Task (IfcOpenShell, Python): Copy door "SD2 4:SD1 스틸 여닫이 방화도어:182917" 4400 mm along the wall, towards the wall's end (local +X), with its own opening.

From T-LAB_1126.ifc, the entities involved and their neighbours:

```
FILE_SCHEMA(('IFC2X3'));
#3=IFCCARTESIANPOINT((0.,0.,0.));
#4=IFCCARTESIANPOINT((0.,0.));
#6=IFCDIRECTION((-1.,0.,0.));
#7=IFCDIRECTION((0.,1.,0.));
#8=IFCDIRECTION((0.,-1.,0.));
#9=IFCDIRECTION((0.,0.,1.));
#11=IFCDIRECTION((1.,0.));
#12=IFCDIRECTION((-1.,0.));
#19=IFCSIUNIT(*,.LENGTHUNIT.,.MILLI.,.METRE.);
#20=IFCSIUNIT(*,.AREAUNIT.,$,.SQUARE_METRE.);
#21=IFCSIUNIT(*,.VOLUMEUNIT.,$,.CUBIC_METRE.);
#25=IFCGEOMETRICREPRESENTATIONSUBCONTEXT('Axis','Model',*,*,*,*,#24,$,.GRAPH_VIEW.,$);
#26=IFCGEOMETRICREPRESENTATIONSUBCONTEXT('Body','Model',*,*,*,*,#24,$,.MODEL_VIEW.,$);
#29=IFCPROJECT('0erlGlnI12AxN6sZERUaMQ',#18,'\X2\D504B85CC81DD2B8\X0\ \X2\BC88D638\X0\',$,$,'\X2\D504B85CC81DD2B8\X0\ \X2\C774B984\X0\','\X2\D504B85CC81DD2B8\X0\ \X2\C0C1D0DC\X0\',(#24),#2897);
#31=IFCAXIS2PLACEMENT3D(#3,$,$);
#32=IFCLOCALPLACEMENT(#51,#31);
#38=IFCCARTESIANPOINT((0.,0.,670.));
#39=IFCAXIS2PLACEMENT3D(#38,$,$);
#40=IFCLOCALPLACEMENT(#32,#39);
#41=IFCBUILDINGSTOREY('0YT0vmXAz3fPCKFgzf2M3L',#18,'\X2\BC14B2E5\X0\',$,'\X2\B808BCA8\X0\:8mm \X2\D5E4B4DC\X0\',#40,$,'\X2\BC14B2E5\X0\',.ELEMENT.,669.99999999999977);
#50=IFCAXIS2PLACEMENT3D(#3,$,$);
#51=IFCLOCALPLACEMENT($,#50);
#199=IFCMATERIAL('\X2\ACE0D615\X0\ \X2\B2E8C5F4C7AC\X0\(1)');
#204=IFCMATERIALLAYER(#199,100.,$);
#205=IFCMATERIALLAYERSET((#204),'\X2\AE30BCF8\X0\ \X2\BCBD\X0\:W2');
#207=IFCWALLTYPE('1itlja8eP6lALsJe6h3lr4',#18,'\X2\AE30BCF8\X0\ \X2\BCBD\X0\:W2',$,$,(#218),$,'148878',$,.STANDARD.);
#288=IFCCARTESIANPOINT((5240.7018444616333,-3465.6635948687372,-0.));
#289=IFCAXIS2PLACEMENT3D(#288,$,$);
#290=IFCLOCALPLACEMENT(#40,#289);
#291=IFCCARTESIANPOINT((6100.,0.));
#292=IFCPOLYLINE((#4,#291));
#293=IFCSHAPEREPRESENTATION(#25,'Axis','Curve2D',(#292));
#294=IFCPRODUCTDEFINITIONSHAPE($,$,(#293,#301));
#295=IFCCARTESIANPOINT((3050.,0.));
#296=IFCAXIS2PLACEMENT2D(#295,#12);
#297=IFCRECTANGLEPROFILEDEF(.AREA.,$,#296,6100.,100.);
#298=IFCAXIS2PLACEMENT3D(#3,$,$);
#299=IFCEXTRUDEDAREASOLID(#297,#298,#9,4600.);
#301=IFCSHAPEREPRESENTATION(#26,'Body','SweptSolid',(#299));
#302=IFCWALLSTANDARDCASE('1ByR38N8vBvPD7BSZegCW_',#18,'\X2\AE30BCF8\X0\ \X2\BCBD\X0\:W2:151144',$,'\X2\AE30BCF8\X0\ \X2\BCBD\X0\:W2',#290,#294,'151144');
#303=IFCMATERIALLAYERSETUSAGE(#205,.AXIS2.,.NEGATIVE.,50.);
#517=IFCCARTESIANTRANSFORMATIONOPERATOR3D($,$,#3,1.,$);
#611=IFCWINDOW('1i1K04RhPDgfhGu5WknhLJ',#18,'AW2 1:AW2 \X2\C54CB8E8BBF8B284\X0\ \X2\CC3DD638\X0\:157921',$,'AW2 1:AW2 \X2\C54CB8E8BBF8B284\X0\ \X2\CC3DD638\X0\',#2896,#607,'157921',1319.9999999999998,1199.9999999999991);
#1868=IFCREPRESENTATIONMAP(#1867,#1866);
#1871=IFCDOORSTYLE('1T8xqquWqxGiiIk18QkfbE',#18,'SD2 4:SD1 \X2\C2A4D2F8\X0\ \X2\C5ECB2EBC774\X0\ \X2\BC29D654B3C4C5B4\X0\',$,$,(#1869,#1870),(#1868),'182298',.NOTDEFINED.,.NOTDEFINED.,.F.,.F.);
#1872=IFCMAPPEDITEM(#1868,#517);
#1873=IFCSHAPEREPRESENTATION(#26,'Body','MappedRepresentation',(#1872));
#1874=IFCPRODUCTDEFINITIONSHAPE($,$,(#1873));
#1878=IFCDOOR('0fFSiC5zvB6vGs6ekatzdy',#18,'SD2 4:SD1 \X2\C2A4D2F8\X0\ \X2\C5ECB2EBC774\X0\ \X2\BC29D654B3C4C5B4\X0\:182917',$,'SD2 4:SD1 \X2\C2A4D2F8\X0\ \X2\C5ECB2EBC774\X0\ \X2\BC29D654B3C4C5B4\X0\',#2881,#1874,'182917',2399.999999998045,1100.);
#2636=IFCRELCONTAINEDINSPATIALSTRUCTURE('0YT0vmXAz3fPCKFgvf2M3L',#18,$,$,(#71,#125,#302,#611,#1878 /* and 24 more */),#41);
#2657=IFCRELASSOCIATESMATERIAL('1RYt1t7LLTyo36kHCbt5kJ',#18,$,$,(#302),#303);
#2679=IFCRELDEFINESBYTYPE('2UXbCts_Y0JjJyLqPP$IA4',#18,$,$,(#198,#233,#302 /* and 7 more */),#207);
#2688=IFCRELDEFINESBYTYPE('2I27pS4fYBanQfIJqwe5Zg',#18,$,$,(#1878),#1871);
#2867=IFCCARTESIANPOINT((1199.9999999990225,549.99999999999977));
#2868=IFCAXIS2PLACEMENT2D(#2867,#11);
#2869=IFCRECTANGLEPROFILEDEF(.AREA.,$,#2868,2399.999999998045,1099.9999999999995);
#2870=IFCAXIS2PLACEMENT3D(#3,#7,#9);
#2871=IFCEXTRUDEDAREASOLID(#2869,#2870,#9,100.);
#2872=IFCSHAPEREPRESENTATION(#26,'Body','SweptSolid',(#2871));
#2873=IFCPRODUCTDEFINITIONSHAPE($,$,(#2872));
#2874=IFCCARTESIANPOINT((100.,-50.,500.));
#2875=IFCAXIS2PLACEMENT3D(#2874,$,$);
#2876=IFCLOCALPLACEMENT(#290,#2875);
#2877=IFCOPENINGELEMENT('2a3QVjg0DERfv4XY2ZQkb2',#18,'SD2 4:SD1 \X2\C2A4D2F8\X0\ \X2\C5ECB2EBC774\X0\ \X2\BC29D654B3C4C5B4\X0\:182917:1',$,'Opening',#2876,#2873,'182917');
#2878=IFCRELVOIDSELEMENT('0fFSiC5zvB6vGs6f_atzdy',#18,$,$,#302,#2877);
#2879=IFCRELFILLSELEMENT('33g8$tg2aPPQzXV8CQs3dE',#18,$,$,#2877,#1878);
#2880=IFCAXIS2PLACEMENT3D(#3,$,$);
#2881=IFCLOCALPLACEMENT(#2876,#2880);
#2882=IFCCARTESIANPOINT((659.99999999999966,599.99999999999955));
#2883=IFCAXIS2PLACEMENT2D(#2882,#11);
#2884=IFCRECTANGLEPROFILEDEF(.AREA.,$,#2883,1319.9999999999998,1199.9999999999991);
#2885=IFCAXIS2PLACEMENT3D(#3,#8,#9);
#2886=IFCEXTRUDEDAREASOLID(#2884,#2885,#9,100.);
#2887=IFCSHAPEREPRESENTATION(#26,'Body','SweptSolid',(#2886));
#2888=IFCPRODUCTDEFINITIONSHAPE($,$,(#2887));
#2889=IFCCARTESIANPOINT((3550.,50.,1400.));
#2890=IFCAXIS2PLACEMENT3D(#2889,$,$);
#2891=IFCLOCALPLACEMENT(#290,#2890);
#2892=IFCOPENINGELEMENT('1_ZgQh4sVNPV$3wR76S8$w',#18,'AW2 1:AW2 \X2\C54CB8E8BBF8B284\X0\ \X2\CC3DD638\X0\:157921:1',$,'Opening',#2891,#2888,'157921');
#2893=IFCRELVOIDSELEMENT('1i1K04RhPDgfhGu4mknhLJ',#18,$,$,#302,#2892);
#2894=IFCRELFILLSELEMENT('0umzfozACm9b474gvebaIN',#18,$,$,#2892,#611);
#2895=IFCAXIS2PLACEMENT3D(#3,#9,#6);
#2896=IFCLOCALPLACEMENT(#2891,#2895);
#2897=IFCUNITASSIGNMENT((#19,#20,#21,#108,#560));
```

```python
import ifcopenshell
import ifcopenshell.api.feature
import ifcopenshell.api.geometry
import ifcopenshell.api.root
import ifcopenshell.geom
import ifcopenshell.util.element
import ifcopenshell.util.placement
import ifcopenshell.util.shape

model = ifcopenshell.open("T-LAB_1126.ifc")
settings = ifcopenshell.geom.settings()


def volume(element):
    """Net volume in cubic metres, openings subtracted."""
    shape = ifcopenshell.geom.create_shape(settings, element)
    return ifcopenshell.util.shape.get_volume(shape.geometry)


def reuse_history(source, copy):
    """copy_class also copies each property set's owner history, people and application; keep the originals."""
    for rel in copy.IsDefinedBy:
        if rel.is_a("IfcRelDefinesByProperties") and (history := rel.RelatingPropertyDefinition.OwnerHistory):
            rel.RelatingPropertyDefinition.OwnerHistory = source.OwnerHistory
            ifcopenshell.util.element.remove_deep2(model, history)


door = model.by_id(1878)
opening = door.FillsVoids[0].RelatingOpeningElement
wall = opening.VoidsElements[0].RelatingBuildingElement
before = volume(wall)
shift = ifcopenshell.util.placement.get_local_placement(wall.ObjectPlacement)[:3, 0] * 4400.0

# copy_class copies the void relationship, type, container and properties, but no geometry.
new_opening = ifcopenshell.api.root.copy_class(model, product=opening)
new_opening.Representation = ifcopenshell.util.element.copy_deep(
    model, opening.Representation, exclude=["IfcGeometricRepresentationContext", "IfcRepresentationMap"]
)
new_opening.Name = "SD2 4:SD1 스틸 여닫이 방화도어"
new_opening.Tag = None
new_door = ifcopenshell.api.root.copy_class(model, product=door)
new_door.Representation = ifcopenshell.util.element.copy_deep(
    model, door.Representation, exclude=["IfcGeometricRepresentationContext", "IfcRepresentationMap"]
)
new_door.Name = "SD2 4:SD1 스틸 여닫이 방화도어"
new_door.Tag = None
reuse_history(door, new_door)
fills = ifcopenshell.api.feature.add_filling(model, opening=new_opening, element=new_door)
fills.OwnerHistory = new_door.OwnerHistory  # required in IFC2X3

for old, new in ((opening, new_opening), (door, new_door)):
    matrix = ifcopenshell.util.placement.get_local_placement(old.ObjectPlacement)
    matrix[:3, 3] += shift
    ifcopenshell.api.geometry.edit_object_placement(model, product=new, matrix=matrix, is_si=False)

after = volume(wall)

print(f"wall volume {before:.3f} -> {after:.3f} m3")

model.write("T-LAB_1126_v2.ifc")
```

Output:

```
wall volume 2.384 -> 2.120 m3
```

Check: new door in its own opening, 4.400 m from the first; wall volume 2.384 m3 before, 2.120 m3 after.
